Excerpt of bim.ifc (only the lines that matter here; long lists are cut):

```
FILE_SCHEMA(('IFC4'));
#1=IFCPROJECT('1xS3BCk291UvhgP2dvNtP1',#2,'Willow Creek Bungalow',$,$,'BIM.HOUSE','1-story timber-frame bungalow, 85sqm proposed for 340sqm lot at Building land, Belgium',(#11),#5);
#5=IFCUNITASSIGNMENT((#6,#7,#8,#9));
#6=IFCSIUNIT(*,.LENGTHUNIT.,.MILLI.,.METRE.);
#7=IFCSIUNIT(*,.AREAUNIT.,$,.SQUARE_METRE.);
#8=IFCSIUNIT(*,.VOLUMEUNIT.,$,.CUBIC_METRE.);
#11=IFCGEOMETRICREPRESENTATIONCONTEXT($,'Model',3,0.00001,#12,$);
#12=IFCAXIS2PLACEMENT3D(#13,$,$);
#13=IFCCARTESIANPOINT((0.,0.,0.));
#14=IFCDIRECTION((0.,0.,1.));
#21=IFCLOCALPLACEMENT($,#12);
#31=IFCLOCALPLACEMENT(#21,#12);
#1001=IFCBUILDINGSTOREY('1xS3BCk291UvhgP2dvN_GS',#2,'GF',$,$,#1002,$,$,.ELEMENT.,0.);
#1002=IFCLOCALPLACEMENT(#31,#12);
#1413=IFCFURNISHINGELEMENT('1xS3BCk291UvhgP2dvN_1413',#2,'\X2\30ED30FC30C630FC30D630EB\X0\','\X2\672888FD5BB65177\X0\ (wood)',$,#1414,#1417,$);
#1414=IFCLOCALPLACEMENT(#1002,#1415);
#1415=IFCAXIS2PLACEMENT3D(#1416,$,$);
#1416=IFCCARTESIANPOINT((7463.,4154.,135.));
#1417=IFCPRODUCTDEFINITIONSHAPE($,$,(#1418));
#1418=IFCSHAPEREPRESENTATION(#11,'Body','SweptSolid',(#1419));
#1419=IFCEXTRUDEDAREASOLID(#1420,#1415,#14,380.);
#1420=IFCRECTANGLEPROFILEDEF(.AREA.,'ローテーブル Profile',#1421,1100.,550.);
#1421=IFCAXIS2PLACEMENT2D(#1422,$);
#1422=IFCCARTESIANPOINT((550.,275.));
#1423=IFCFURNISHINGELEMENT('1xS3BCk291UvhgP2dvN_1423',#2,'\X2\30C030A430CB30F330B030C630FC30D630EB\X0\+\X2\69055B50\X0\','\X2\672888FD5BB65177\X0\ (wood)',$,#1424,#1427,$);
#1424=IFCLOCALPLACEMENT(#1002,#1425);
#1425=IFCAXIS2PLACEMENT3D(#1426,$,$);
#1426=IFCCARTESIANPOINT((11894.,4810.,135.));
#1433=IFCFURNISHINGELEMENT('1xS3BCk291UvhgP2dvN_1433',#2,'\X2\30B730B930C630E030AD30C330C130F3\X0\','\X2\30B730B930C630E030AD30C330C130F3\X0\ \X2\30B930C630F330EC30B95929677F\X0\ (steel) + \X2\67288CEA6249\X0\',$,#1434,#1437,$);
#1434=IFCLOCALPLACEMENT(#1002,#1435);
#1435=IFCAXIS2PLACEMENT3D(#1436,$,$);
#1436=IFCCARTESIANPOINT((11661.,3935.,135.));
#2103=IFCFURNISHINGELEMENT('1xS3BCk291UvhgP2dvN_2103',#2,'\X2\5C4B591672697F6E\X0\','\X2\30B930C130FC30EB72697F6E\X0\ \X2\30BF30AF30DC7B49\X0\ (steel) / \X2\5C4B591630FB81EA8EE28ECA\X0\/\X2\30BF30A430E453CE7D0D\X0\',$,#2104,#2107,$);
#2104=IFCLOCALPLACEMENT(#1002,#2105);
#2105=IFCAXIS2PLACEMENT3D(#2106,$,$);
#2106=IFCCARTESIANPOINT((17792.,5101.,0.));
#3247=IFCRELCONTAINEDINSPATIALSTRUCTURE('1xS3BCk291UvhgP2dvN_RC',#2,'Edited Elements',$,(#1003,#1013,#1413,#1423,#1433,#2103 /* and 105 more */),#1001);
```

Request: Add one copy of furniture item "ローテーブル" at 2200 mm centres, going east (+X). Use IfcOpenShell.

```python
import numpy as np
import ifcopenshell
import ifcopenshell.api.geometry
import ifcopenshell.api.root
import ifcopenshell.util.element
import ifcopenshell.util.placement
import ifcopenshell.util.unit

model = ifcopenshell.open("bim.ifc")
unit_scale = ifcopenshell.util.unit.calculate_unit_scale(model)


def reuse_history(source, copy):
    """copy_class also copies each property set's owner history, people and application; keep the originals."""
    for rel in copy.IsDefinedBy:
        if rel.is_a("IfcRelDefinesByProperties") and (history := rel.RelatingPropertyDefinition.OwnerHistory):
            rel.RelatingPropertyDefinition.OwnerHistory = source.OwnerHistory
            ifcopenshell.util.element.remove_deep2(model, history)


source = model.by_guid("1xS3BCk291UvhgP2dvN_1413")
base = ifcopenshell.util.placement.get_local_placement(source.ObjectPlacement)
step = np.array([1.0, 0.0, 0.0]) * 2.2 / unit_scale

for i in range(1, 2):
    copy = ifcopenshell.api.root.copy_class(model, product=source)
    copy.Representation = ifcopenshell.util.element.copy_deep(
        model, source.Representation, exclude=["IfcGeometricRepresentationContext", "IfcRepresentationMap"]
    )
    reuse_history(source, copy)
    matrix = base.copy()
    matrix[:3, 3] += i * step
    print("added at", matrix[:3, 3].round(3) + 0.0)
    ifcopenshell.api.geometry.edit_object_placement(model, product=copy, matrix=matrix, is_si=False)

model.write("bim_edited.ifc")
```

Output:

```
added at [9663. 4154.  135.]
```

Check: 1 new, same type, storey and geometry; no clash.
